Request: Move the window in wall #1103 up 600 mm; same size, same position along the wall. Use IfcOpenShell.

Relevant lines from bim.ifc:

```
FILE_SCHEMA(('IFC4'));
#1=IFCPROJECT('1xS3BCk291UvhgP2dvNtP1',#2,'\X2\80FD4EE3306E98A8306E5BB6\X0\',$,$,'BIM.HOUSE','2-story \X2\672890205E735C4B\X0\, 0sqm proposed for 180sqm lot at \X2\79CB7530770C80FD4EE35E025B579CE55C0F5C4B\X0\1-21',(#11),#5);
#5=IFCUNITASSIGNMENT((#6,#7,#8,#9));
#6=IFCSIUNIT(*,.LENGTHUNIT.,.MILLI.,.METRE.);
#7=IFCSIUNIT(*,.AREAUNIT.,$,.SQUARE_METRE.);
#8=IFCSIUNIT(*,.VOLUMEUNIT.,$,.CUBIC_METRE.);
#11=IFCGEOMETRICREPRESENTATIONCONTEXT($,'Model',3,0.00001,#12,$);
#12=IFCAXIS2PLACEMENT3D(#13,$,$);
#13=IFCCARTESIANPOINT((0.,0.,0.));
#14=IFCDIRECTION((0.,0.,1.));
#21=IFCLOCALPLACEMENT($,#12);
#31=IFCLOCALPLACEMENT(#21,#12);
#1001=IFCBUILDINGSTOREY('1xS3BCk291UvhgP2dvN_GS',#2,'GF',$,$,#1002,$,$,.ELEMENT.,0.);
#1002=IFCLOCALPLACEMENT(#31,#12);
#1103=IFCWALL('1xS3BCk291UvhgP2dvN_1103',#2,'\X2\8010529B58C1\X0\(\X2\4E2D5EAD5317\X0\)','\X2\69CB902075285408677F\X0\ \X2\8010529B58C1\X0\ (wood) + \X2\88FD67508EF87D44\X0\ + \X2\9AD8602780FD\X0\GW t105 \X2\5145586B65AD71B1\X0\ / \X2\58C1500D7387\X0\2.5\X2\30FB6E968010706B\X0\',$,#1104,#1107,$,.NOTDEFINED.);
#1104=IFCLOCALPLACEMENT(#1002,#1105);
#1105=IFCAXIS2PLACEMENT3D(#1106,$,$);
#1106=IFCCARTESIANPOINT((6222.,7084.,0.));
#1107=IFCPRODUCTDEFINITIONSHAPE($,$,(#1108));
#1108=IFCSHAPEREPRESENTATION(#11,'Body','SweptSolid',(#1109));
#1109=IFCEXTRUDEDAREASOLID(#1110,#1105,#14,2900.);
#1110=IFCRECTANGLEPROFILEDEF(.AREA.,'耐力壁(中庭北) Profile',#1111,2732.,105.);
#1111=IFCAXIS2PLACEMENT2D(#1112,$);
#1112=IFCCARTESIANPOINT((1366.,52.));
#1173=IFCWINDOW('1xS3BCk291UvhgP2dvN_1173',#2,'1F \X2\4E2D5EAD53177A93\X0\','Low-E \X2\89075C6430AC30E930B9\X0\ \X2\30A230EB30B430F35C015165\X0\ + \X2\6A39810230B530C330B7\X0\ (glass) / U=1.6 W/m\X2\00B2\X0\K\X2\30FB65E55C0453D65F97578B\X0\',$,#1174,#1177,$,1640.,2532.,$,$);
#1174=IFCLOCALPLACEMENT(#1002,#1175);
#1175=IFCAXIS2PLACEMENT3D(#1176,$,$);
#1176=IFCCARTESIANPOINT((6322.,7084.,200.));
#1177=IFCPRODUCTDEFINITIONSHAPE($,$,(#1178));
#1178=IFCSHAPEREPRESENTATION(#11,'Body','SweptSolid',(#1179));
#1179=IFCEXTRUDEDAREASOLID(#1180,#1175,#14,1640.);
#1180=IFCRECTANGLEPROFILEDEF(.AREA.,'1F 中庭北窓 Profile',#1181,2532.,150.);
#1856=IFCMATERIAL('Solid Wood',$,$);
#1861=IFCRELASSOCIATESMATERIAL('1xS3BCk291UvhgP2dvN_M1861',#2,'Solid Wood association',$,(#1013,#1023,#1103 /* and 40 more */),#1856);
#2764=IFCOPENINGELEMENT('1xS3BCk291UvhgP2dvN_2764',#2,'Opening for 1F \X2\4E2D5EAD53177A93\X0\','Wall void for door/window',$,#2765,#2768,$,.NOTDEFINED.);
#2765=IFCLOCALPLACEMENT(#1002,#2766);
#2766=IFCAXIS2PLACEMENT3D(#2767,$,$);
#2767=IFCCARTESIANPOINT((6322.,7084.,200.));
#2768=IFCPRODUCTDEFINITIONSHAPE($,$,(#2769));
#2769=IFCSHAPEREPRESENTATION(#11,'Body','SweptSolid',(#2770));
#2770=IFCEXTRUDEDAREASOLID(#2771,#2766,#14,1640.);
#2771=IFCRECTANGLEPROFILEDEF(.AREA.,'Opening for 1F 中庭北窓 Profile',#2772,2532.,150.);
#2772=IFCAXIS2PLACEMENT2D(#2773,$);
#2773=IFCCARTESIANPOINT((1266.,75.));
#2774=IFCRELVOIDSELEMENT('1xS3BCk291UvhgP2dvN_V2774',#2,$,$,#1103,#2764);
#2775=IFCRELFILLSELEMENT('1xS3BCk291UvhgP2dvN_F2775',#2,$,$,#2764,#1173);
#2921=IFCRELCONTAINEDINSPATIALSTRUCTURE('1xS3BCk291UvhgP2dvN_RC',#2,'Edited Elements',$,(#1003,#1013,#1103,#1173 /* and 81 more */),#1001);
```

```python
import numpy as np
import ifcopenshell
import ifcopenshell.api.geometry
import ifcopenshell.util.placement
import ifcopenshell.util.unit

model = ifcopenshell.open("bim.ifc")
unit_scale = ifcopenshell.util.unit.calculate_unit_scale(model)

window = model.by_guid("1xS3BCk291UvhgP2dvN_1173")
opening = window.FillsVoids[0].RelatingOpeningElement
dz = 0.6 / unit_scale

shift = np.array([0.0, 0.0, dz])
# The window is not placed relative to its opening, so move both.
for product in (opening, window):
    matrix = ifcopenshell.util.placement.get_local_placement(product.ObjectPlacement)
    matrix[:3, 3] += shift
    ifcopenshell.api.geometry.edit_object_placement(model, product=product, matrix=matrix, is_si=False)

print(f"moved by {dz * unit_scale:+.3f} m")

model.write("bim_v2.ifc")
```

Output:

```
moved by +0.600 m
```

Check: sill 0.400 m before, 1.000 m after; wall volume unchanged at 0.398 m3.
